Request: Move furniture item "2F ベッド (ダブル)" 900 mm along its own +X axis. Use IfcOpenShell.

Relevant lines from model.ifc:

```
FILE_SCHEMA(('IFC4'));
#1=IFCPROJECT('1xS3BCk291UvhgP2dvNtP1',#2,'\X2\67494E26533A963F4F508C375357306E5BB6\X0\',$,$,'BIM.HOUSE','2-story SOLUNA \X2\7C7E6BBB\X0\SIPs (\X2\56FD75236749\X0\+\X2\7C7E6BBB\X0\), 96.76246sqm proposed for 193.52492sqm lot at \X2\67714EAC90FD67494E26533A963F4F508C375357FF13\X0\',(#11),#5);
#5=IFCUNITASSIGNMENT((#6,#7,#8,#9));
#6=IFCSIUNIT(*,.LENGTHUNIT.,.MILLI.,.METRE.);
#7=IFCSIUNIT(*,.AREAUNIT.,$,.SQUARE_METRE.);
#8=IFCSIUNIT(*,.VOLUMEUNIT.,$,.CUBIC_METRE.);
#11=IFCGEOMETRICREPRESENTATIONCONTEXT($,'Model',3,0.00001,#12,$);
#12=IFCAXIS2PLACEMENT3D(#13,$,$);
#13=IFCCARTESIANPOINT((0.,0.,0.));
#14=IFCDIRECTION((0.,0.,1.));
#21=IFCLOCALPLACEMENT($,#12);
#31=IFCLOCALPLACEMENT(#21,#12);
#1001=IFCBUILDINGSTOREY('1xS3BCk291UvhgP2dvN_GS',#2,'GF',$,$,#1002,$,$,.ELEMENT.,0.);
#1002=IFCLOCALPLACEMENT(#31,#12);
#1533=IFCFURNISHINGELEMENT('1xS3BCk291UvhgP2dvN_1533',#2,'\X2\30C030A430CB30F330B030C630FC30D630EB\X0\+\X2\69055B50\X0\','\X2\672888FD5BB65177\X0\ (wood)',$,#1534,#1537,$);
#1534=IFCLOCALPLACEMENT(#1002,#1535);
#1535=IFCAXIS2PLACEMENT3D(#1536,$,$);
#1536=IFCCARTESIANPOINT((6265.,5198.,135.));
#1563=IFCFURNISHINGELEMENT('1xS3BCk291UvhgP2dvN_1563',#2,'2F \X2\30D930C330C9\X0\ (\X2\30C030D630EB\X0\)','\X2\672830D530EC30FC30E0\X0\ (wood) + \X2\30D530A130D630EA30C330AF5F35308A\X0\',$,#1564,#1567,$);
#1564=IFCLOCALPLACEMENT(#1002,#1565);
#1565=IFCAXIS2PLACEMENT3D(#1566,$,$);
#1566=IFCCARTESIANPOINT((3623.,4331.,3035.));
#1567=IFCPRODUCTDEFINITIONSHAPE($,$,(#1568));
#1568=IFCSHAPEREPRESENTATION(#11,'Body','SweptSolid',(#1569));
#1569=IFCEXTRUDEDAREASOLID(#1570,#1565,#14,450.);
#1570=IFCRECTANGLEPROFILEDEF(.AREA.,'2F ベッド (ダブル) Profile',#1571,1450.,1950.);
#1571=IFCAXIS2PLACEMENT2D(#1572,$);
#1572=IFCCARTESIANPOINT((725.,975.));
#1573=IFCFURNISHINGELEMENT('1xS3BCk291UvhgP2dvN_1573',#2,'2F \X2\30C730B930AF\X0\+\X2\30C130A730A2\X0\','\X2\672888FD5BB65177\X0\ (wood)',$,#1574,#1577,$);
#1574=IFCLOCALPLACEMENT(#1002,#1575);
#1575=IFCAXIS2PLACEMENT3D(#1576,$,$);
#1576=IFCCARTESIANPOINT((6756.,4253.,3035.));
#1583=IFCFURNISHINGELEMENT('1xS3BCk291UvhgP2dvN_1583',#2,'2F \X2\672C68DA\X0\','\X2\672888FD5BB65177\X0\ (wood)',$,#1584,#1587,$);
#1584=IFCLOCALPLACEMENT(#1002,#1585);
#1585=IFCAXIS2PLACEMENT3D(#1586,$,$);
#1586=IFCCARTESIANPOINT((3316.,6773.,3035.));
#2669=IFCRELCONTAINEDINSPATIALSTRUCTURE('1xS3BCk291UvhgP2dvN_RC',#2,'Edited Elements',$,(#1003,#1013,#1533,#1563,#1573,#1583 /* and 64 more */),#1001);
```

```python
import ifcopenshell
import ifcopenshell.api.geometry
import ifcopenshell.util.placement

model = ifcopenshell.open("model.ifc")

item = model.by_id(1563)
matrix = ifcopenshell.util.placement.get_local_placement(item.ObjectPlacement)
matrix[:3, 3] += matrix[:3, 0] * 900.0
ifcopenshell.api.geometry.edit_object_placement(model, product=item, matrix=matrix, is_si=False)

print(ifcopenshell.util.placement.get_local_placement(item.ObjectPlacement).round(3) + 0.0)

model.write("model_v2.ifc")
```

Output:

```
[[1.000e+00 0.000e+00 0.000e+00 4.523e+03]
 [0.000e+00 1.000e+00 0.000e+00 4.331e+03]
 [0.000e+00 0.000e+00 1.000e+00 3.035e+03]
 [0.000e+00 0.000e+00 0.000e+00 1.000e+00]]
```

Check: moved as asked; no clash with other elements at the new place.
